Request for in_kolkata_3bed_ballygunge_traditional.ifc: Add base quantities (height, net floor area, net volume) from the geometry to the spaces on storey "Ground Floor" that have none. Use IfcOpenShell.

First a look at what the model holds.

```python
import ifcopenshell
import ifcopenshell.util.element
import ifcopenshell.util.unit

model = ifcopenshell.open("in_kolkata_3bed_ballygunge_traditional.ifc")
print(model.schema)
for unit_type in ("LENGTHUNIT", "AREAUNIT", "VOLUMEUNIT"):
    print(unit_type, ifcopenshell.util.unit.calculate_unit_scale(model, unit_type))
storey = next(s for s in model.by_type("IfcBuildingStorey") if s.Name == "Ground Floor")
spaces = [e for e in ifcopenshell.util.element.get_decomposition(storey) if e.is_a("IfcSpace")]
for e in sorted(spaces, key=lambda e: e.id()):
    print(e.id(), e.is_a(), e.Name, list(ifcopenshell.util.element.get_psets(e, qtos_only=True)), sep=" | ")
```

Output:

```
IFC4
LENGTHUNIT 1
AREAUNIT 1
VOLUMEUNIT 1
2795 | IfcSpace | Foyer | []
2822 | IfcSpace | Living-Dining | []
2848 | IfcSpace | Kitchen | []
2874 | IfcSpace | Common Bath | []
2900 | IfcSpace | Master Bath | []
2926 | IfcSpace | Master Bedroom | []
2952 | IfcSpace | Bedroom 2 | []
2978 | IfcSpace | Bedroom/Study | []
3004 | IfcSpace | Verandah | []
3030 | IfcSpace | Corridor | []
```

```python
import ifcopenshell
import ifcopenshell.api.pset
import ifcopenshell.geom
import ifcopenshell.util.element
import ifcopenshell.util.shape
import ifcopenshell.util.unit

model = ifcopenshell.open("in_kolkata_3bed_ballygunge_traditional.ifc")
unit_scale = ifcopenshell.util.unit.calculate_unit_scale(model)
area_scale = ifcopenshell.util.unit.calculate_unit_scale(model, "AREAUNIT")
volume_scale = ifcopenshell.util.unit.calculate_unit_scale(model, "VOLUMEUNIT")
settings = ifcopenshell.geom.settings()

storey = next(s for s in model.by_type("IfcBuildingStorey") if s.Name == "Ground Floor")
spaces = [e for e in ifcopenshell.util.element.get_decomposition(storey) if e.is_a("IfcSpace")]

for e in sorted(spaces, key=lambda e: e.id()):
    if ifcopenshell.util.element.get_psets(e, qtos_only=True, should_inherit=False):
        continue
    # Geometry comes back in metres, in the element's own axes.
    shape = ifcopenshell.geom.create_shape(settings, e)
    values = {
        "Height": ifcopenshell.util.shape.get_z(shape.geometry) / unit_scale,
        "NetFloorArea": ifcopenshell.util.shape.get_footprint_area(shape.geometry) / area_scale,
        "NetVolume": ifcopenshell.util.shape.get_volume(shape.geometry) / volume_scale,
    }
    qto = ifcopenshell.api.pset.add_qto(model, product=e, name="Qto_SpaceBaseQuantities")
    ifcopenshell.api.pset.edit_qto(model, qto=qto, properties=values)
    print(e.id(), {k: round(v, 3) for k, v in values.items()})

model.write("in_kolkata_3bed_ballygunge_traditional-out.ifc")
```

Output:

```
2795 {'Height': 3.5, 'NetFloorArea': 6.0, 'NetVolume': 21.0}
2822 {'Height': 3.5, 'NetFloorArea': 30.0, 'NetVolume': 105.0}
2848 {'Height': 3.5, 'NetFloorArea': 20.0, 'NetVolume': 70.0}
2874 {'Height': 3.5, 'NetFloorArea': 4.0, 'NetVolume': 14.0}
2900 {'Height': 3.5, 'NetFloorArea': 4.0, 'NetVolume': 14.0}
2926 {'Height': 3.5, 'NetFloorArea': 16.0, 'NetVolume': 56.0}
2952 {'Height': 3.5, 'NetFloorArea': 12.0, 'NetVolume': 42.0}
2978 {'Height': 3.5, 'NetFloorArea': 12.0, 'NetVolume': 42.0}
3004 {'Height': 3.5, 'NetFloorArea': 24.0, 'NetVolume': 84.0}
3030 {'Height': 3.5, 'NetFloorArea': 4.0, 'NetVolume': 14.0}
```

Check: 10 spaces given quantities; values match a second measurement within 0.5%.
